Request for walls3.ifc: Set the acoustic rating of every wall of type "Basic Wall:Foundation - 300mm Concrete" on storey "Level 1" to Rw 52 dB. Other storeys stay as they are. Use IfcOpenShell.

First a look at what the model holds.

```python
import ifcopenshell
import ifcopenshell.util.element

model = ifcopenshell.open("walls3.ifc")
print(model.schema)
storey = next(s for s in model.by_type("IfcBuildingStorey") if s.Name == "Level 1")
walls = [e for e in ifcopenshell.util.element.get_decomposition(storey) if e.is_a("IfcWall")]
seen = {}
for e in walls:
    element_type = ifcopenshell.util.element.get_type(e)
    key = (element_type.Name if element_type != e and element_type else None, ifcopenshell.util.element.get_pset(e, "Pset_WallCommon", "AcousticRating"))
    seen[key] = seen.get(key, 0) + 1
for (name, value), count in sorted(seen.items(), key=str):
    print(count, "x", name, "|", value)
```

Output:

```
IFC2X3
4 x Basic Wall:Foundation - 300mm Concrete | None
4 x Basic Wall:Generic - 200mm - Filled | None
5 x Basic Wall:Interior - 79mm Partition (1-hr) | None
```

```python
import ifcopenshell
import ifcopenshell.api.pset
import ifcopenshell.util.element

model = ifcopenshell.open("walls3.ifc")

storey = next(s for s in model.by_type("IfcBuildingStorey") if s.Name == "Level 1")
walls = [e for e in ifcopenshell.util.element.get_decomposition(storey) if e.is_a("IfcWall")]

count = 0
for e in walls:
    element_type = ifcopenshell.util.element.get_type(e)
    if element_type in (None, e) or element_type.Name != "Basic Wall:Foundation - 300mm Concrete":
        continue
    # add_pset returns the element's existing set when there is one.
    pset = ifcopenshell.api.pset.add_pset(model, product=e, name="Pset_WallCommon")
    ifcopenshell.api.pset.edit_pset(model, pset=pset, properties={"AcousticRating": "Rw 52 dB"})
    count += 1

print(count, "walls updated")

model.write("walls3_updated.ifc")
```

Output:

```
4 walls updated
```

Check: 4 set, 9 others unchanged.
